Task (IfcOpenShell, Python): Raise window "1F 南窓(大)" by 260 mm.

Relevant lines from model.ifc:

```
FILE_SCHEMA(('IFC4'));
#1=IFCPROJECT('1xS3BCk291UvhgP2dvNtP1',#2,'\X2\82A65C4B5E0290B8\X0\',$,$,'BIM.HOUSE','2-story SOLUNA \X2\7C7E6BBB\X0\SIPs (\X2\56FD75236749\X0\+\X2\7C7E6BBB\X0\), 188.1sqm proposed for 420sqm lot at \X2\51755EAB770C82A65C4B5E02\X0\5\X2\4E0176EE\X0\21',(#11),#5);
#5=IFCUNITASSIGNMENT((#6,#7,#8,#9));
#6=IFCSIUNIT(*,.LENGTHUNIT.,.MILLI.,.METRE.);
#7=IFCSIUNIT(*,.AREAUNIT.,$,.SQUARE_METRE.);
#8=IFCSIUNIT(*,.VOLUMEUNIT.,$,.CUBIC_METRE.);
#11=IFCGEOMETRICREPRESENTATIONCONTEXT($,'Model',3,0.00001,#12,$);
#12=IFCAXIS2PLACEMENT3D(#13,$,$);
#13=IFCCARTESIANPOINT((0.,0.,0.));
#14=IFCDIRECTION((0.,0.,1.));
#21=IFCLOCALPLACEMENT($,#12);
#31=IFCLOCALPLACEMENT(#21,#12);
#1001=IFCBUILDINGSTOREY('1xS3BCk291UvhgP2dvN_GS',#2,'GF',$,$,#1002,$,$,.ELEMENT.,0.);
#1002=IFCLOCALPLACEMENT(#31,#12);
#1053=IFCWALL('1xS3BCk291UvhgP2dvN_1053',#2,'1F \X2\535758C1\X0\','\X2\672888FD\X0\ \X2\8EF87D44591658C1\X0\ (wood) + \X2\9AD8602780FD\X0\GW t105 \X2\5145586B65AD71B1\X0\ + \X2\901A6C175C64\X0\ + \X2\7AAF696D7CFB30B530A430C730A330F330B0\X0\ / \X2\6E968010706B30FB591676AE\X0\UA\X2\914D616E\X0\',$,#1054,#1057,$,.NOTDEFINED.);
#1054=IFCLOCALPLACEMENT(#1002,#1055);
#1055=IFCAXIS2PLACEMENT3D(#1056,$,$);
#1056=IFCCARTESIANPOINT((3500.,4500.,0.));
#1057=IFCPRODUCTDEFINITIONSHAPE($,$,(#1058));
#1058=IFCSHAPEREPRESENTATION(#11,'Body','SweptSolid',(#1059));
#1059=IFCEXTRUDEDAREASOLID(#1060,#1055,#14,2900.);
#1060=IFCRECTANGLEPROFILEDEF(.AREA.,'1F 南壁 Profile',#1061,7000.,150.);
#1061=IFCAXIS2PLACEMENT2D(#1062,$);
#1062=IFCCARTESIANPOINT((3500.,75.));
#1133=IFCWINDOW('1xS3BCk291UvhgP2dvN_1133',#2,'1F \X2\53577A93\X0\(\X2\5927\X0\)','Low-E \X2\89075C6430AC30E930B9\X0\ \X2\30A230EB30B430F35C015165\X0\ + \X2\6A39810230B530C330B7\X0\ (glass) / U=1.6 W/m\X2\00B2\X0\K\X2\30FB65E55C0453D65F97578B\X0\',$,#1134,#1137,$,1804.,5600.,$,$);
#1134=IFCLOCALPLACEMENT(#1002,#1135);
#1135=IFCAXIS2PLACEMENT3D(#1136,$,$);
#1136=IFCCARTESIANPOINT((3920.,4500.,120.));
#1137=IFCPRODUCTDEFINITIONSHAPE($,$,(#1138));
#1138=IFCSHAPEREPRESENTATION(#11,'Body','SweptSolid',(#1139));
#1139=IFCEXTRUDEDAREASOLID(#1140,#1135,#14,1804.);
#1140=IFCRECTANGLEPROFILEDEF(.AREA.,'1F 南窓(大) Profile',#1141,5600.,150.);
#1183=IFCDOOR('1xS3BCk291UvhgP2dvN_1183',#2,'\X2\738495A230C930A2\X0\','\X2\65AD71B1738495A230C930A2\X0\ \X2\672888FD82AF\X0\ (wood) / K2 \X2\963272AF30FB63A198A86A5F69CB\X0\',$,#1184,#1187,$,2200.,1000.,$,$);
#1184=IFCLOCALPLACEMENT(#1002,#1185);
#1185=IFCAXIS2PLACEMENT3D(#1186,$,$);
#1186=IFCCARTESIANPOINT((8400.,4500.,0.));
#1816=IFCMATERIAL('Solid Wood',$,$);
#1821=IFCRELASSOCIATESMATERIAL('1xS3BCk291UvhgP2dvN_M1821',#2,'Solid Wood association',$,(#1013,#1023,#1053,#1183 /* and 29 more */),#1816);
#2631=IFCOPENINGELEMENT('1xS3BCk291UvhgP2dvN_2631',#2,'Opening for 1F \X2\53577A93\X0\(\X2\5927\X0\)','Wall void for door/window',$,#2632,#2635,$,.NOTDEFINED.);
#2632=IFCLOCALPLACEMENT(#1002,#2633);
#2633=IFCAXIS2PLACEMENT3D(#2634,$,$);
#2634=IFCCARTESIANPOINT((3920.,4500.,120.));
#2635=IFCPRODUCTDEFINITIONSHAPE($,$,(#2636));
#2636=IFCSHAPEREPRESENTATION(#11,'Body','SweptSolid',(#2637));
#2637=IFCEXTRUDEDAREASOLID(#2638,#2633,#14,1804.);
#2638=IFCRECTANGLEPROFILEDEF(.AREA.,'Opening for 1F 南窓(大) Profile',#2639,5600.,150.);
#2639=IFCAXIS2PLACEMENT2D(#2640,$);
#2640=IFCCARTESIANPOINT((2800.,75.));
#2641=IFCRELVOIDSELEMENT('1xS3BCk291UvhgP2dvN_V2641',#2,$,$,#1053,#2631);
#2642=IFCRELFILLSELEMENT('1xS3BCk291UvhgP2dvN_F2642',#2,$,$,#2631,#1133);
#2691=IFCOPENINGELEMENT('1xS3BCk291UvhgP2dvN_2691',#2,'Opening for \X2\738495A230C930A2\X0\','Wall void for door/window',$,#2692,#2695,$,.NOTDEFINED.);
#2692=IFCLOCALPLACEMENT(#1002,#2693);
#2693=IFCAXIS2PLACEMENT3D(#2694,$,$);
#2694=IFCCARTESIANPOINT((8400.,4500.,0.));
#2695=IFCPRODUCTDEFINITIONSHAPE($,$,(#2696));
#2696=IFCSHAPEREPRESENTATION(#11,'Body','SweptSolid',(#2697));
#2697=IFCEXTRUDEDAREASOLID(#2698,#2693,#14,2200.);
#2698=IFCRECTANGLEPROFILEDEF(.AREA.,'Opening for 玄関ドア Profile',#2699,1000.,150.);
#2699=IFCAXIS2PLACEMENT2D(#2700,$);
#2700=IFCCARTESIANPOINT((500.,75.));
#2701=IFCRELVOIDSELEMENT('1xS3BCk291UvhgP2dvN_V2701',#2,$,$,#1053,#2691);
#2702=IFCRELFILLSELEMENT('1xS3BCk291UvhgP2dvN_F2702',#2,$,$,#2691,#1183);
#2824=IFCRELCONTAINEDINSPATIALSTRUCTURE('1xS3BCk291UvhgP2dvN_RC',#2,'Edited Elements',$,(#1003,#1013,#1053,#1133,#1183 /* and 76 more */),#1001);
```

```python
import numpy as np
import ifcopenshell
import ifcopenshell.api.geometry
import ifcopenshell.util.placement
import ifcopenshell.util.unit

model = ifcopenshell.open("model.ifc")
unit_scale = ifcopenshell.util.unit.calculate_unit_scale(model)

window = model.by_guid("1xS3BCk291UvhgP2dvN_1133")
opening = window.FillsVoids[0].RelatingOpeningElement
dz = 0.26 / unit_scale

shift = np.array([0.0, 0.0, dz])
# The window is not placed relative to its opening, so move both.
for product in (opening, window):
    matrix = ifcopenshell.util.placement.get_local_placement(product.ObjectPlacement)
    matrix[:3, 3] += shift
    ifcopenshell.api.geometry.edit_object_placement(model, product=product, matrix=matrix, is_si=False)

print(f"moved by {dz * unit_scale:+.3f} m")

model.write("model_rev.ifc")
```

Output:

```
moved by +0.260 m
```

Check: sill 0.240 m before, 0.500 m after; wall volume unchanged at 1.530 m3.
